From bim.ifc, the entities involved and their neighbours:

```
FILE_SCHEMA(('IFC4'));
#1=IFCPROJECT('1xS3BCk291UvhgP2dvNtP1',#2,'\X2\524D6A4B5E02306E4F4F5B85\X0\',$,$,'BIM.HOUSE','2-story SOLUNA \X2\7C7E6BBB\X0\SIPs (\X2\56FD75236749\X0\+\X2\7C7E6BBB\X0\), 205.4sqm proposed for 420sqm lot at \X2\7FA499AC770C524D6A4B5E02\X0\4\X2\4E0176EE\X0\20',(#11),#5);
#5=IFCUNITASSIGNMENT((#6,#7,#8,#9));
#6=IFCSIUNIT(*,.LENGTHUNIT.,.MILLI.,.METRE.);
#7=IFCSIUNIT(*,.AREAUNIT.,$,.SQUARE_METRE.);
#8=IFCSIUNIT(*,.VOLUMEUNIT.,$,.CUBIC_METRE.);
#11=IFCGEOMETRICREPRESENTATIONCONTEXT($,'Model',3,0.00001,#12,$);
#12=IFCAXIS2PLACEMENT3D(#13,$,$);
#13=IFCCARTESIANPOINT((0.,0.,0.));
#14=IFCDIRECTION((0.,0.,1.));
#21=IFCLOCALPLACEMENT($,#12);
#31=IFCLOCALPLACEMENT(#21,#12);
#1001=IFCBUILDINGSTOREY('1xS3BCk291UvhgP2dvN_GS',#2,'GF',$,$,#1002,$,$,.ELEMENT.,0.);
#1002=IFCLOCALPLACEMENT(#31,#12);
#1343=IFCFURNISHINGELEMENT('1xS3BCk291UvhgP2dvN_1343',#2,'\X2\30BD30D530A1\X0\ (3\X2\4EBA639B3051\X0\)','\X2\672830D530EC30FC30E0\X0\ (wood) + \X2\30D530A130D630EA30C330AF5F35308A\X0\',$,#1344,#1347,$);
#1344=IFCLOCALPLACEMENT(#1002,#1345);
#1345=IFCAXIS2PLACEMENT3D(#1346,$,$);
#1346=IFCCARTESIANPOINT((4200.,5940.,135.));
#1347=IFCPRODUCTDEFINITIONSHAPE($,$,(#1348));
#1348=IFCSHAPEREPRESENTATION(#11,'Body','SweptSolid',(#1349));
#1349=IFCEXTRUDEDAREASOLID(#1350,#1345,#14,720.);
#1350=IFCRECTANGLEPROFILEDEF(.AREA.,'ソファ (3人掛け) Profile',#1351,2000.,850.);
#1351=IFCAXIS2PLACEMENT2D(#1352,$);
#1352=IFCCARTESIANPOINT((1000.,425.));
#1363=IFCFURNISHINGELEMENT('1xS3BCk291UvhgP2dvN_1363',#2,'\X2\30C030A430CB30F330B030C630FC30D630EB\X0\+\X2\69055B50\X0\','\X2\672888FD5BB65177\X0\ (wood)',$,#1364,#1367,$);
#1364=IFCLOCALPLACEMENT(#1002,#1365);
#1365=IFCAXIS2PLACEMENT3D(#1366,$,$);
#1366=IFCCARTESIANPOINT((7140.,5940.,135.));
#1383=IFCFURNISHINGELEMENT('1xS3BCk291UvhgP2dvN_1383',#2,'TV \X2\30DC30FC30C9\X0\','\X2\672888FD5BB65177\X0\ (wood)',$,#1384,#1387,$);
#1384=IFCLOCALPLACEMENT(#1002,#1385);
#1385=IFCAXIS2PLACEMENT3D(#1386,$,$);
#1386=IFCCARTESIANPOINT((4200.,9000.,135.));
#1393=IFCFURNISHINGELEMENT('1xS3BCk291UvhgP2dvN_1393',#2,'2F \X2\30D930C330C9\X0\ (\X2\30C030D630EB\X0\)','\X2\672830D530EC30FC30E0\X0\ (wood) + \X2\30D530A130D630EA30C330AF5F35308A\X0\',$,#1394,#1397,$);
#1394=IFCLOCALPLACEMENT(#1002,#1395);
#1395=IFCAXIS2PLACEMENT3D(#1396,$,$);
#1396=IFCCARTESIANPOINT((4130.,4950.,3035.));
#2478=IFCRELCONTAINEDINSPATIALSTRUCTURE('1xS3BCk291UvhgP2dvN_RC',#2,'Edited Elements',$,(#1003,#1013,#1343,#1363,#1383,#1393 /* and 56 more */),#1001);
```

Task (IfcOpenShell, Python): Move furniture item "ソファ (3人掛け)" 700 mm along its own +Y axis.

```python
import ifcopenshell
import ifcopenshell.api.geometry
import ifcopenshell.util.placement

model = ifcopenshell.open("bim.ifc")

item = model.by_guid("1xS3BCk291UvhgP2dvN_1343")
matrix = ifcopenshell.util.placement.get_local_placement(item.ObjectPlacement)
matrix[:3, 3] += matrix[:3, 1] * 700.0
ifcopenshell.api.geometry.edit_object_placement(model, product=item, matrix=matrix, is_si=False)

print(ifcopenshell.util.placement.get_local_placement(item.ObjectPlacement).round(3) + 0.0)

model.write("bim_updated.ifc")
```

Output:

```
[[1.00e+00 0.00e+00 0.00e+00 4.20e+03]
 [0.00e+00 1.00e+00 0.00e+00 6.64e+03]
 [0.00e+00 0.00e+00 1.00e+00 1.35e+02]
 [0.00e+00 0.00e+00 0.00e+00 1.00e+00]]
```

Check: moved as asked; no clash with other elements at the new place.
